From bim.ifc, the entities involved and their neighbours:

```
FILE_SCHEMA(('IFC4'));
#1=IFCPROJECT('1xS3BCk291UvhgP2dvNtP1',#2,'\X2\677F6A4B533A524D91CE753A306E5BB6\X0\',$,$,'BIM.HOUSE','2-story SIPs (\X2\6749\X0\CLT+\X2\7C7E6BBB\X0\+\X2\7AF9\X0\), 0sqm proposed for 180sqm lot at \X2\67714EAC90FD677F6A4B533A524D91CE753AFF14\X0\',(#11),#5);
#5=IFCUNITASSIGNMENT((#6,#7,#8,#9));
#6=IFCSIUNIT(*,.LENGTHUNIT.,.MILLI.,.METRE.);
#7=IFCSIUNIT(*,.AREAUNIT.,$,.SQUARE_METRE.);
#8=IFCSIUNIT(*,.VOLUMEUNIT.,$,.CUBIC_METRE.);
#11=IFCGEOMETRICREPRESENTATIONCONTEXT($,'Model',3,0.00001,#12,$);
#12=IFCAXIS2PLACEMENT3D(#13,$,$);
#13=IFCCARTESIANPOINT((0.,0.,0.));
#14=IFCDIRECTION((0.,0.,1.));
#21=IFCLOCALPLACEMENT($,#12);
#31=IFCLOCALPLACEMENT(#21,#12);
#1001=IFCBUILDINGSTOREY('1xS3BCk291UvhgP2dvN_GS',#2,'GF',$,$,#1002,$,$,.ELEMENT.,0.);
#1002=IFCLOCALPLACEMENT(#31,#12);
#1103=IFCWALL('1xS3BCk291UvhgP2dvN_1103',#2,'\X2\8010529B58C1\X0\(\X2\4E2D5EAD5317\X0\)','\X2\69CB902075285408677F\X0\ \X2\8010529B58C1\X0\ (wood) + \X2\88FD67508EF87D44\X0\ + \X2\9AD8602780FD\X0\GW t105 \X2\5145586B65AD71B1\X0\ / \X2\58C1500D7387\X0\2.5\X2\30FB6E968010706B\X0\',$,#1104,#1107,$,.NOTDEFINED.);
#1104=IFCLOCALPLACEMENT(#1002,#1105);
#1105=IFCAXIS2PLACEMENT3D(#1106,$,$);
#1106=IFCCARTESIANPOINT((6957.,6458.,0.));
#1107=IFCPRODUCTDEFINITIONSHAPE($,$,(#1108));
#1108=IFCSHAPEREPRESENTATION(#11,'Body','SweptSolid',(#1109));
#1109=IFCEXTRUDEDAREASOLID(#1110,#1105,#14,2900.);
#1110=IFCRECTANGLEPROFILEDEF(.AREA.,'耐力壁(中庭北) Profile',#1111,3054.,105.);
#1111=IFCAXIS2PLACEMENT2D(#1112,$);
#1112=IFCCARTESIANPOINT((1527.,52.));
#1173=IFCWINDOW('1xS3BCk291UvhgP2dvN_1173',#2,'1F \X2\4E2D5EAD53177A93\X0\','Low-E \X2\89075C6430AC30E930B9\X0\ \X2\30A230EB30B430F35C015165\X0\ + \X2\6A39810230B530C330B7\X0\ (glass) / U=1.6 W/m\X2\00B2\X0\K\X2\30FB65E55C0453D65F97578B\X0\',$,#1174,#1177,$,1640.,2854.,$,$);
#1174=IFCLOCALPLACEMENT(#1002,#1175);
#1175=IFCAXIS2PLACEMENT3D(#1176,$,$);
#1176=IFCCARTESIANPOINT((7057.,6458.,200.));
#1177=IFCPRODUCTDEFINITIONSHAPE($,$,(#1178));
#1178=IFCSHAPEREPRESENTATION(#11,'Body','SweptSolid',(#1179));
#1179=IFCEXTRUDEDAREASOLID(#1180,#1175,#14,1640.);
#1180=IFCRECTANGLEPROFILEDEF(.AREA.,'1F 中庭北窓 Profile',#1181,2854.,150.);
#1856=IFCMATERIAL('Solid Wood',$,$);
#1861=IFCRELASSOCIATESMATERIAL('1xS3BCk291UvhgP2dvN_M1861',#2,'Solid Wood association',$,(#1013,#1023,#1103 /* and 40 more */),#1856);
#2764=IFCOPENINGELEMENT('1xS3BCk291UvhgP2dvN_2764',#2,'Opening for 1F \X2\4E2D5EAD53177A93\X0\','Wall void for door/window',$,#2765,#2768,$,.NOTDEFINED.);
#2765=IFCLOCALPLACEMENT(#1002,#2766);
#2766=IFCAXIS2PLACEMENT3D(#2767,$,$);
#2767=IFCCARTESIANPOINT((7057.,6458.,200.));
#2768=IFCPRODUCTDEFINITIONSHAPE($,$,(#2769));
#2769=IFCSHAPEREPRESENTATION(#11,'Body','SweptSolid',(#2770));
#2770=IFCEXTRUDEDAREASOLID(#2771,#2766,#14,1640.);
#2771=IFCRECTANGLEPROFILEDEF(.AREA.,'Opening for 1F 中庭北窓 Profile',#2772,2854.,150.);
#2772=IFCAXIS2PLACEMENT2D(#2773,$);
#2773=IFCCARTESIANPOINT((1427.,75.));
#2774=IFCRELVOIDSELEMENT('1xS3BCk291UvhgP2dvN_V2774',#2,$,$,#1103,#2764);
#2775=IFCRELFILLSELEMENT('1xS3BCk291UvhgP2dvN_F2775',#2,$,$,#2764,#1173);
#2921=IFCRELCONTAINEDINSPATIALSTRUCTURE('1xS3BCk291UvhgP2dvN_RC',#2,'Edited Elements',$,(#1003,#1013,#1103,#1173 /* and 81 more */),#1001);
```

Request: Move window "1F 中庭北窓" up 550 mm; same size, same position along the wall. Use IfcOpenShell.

```python
import numpy as np
import ifcopenshell
import ifcopenshell.api.geometry
import ifcopenshell.util.placement
import ifcopenshell.util.unit

model = ifcopenshell.open("bim.ifc")
unit_scale = ifcopenshell.util.unit.calculate_unit_scale(model)

window = model.by_id(1173)
opening = window.FillsVoids[0].RelatingOpeningElement
dz = 550.0

shift = np.array([0.0, 0.0, dz])
# The window is not placed relative to its opening, so move both.
for product in (opening, window):
    matrix = ifcopenshell.util.placement.get_local_placement(product.ObjectPlacement)
    matrix[:3, 3] += shift
    ifcopenshell.api.geometry.edit_object_placement(model, product=product, matrix=matrix, is_si=False)

print(f"moved by {dz * unit_scale:+.3f} m")

model.write("bim-out.ifc")
```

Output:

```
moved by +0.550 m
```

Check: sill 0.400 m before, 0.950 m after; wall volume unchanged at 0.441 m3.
